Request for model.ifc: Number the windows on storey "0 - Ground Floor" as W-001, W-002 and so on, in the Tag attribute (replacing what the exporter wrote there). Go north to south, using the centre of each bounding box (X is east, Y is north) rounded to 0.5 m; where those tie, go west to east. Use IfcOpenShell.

First a look at what the model holds.

```python
import ifcopenshell
import ifcopenshell.util.element
import ifcopenshell.util.placement

model = ifcopenshell.open("model.ifc")
print(model.schema)
storey = next(s for s in model.by_type("IfcBuildingStorey") if s.Name == "0 - Ground Floor")
windows = [e for e in ifcopenshell.util.element.get_decomposition(storey) if e.is_a("IfcWindow")]
for e in sorted(windows, key=lambda e: e.id()):
    origin = ifcopenshell.util.placement.get_local_placement(e.ObjectPlacement)[:3, 3]
    print(e.id(), e.Tag, e.Name, origin.round(2) + 0.0, sep=" | ")
```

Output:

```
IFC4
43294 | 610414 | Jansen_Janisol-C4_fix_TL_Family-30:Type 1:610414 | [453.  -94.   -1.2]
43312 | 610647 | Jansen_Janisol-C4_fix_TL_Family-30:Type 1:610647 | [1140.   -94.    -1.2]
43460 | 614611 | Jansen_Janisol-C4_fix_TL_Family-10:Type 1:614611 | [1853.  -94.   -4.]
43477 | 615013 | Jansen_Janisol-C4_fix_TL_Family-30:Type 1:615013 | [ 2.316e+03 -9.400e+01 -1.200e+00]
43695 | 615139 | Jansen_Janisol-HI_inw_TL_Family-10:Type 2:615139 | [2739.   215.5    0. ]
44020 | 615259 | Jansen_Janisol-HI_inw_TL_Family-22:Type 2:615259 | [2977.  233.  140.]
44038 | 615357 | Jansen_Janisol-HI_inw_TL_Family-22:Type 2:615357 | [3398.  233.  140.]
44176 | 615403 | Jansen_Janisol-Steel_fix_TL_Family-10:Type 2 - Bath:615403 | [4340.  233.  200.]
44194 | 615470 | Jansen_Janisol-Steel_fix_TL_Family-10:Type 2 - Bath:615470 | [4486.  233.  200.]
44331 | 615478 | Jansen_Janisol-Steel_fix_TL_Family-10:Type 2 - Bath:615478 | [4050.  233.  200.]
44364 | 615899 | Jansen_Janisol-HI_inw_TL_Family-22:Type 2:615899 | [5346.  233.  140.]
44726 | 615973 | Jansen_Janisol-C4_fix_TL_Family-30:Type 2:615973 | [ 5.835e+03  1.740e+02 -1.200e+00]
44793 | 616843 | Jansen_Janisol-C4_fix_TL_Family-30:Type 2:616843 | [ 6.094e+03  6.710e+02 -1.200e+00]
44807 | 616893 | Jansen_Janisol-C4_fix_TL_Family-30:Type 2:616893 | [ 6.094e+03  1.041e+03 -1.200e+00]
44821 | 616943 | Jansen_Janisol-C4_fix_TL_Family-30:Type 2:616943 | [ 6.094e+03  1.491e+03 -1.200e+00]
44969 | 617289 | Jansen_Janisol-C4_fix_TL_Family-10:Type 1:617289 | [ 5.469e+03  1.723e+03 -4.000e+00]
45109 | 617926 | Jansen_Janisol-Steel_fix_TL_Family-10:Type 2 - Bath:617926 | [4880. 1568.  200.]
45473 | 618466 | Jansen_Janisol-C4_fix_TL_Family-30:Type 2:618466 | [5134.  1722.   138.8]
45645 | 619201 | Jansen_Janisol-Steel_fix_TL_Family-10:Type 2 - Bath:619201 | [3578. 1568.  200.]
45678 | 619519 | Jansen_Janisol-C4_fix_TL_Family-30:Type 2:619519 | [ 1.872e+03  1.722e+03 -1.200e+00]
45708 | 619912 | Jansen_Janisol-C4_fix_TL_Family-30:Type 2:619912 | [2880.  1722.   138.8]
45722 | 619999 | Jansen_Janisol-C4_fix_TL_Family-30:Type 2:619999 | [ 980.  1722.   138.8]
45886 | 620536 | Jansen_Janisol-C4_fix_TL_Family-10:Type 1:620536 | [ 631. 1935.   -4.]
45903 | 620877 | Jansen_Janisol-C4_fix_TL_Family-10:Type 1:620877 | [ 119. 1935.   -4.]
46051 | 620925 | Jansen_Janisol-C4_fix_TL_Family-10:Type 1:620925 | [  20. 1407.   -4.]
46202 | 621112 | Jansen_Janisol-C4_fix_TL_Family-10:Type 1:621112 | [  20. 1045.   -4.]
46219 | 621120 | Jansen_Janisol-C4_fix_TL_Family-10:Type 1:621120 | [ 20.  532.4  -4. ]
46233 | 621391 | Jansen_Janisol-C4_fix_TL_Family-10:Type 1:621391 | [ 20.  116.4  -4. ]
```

```python
import ifcopenshell
import ifcopenshell.geom
import ifcopenshell.util.element
import ifcopenshell.util.shape

model = ifcopenshell.open("model.ifc")
settings = ifcopenshell.geom.settings()
settings.set("use-world-coords", True)


def centre(element):
    shape = ifcopenshell.geom.create_shape(settings, element)
    return ifcopenshell.util.shape.get_bbox_centroid(shape.geometry)


storey = next(s for s in model.by_type("IfcBuildingStorey") if s.Name == "0 - Ground Floor")
windows = [e for e in ifcopenshell.util.element.get_decomposition(storey) if e.is_a("IfcWindow")]

# Insertion points can sit at a corner or the storey origin, so sort by the geometry (in metres).
centres = {e: centre(e) for e in windows}
windows.sort(key=lambda e: (-round(centres[e][1] / 0.5), centres[e][0]))

for i, e in enumerate(windows, start=1):
    number = f"W-0{i:02d}"
    e.Tag = number
    print(e.id(), number)

model.write("model_rev.ifc")
```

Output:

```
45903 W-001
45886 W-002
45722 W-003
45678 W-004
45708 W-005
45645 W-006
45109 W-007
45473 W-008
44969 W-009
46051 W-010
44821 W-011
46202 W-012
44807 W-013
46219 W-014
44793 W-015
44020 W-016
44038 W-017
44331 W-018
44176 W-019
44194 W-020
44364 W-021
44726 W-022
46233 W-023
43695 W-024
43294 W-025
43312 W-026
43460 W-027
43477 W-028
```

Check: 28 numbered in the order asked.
